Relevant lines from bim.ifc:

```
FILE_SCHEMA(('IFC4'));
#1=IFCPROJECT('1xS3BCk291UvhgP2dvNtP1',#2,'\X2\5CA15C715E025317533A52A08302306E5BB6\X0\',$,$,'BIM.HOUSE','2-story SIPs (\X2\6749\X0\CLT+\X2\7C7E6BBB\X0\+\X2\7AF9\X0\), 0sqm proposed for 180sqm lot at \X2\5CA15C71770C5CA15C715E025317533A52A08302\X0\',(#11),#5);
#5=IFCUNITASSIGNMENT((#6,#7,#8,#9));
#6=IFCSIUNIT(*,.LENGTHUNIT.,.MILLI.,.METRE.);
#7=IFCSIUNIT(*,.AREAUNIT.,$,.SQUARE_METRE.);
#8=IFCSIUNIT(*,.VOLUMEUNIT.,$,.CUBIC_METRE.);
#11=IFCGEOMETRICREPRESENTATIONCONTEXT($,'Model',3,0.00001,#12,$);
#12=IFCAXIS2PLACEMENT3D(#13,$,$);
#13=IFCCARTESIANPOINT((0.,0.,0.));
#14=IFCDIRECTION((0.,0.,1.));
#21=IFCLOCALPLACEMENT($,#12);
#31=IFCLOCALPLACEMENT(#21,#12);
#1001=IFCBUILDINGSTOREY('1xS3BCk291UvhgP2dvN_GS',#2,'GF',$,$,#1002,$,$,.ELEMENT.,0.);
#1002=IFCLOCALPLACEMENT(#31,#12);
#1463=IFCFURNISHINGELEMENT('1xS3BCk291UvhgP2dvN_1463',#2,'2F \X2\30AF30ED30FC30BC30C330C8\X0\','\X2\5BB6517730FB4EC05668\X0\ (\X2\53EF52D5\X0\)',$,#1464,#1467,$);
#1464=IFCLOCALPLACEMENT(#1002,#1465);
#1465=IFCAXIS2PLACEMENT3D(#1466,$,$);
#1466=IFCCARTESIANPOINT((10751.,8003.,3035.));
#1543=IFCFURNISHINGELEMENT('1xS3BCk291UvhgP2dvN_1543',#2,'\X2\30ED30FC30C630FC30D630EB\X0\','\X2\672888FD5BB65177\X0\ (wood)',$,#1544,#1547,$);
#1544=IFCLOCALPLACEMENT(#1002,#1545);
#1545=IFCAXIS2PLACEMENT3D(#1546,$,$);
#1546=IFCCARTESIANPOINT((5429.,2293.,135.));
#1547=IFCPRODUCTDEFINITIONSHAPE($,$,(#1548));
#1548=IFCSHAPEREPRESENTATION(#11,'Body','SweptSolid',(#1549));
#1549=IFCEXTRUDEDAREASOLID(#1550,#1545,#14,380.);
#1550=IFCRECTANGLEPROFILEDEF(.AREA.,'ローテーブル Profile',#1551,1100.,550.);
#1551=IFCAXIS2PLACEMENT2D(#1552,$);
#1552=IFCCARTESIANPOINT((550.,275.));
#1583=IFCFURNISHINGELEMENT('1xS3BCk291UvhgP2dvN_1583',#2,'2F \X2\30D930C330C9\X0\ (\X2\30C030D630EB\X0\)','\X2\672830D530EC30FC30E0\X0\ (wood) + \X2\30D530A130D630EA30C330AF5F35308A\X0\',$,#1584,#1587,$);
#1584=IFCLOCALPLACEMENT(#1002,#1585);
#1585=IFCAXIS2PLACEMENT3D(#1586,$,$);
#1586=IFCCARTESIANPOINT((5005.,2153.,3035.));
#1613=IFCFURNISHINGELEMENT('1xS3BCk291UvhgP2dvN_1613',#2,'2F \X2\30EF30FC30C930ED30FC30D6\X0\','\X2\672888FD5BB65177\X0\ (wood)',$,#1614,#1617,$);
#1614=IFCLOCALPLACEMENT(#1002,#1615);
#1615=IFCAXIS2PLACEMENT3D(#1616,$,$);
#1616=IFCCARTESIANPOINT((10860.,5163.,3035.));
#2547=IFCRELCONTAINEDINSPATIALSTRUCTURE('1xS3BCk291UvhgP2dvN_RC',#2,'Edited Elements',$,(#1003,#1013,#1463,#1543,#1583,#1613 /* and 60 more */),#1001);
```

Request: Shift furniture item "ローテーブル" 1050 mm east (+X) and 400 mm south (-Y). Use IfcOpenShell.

```python
import ifcopenshell
import ifcopenshell.api.geometry
import ifcopenshell.util.placement
import ifcopenshell.util.unit

model = ifcopenshell.open("bim.ifc")
unit_scale = ifcopenshell.util.unit.calculate_unit_scale(model)

item = model.by_guid("1xS3BCk291UvhgP2dvN_1543")
matrix = ifcopenshell.util.placement.get_local_placement(item.ObjectPlacement)
matrix[0, 3] += 1.05 / unit_scale
matrix[1, 3] -= 0.4 / unit_scale
ifcopenshell.api.geometry.edit_object_placement(model, product=item, matrix=matrix, is_si=False)

print(ifcopenshell.util.placement.get_local_placement(item.ObjectPlacement).round(3) + 0.0)

model.write("bim_updated.ifc")
```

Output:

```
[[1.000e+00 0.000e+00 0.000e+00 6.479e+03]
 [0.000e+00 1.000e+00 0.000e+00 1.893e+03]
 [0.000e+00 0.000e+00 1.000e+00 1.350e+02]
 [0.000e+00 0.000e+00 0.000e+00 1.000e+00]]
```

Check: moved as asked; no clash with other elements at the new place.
